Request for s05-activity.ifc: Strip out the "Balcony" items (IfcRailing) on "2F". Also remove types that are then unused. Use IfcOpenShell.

First a look at what the model holds.

```python
import ifcopenshell
import ifcopenshell.util.element

model = ifcopenshell.open("s05-activity.ifc")
print(model.schema)
storey = next(s for s in model.by_type("IfcBuildingStorey") if s.Name == "2F")
railings = [e for e in ifcopenshell.util.element.get_decomposition(storey) if e.is_a("IfcRailing")]
seen = {}
for e in railings:
    element_type = ifcopenshell.util.element.get_type(e)
    name = element_type.Name if element_type not in (None, e) else None
    seen[name] = seen.get(name, 0) + 1
for name, count in sorted(seen.items(), key=str):
    print(count, "x", name)
```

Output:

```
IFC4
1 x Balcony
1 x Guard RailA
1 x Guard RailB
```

```python
import ifcopenshell
import ifcopenshell.api.root
import ifcopenshell.util.element

model = ifcopenshell.open("s05-activity.ifc")

storey = next(s for s in model.by_type("IfcBuildingStorey") if s.Name == "2F")
railings = [e for e in ifcopenshell.util.element.get_decomposition(storey) if e.is_a("IfcRailing")]
targets = [e for e in railings if (t := ifcopenshell.util.element.get_type(e)) not in (None, e) and t.Name == "Balcony"]
types = {ifcopenshell.util.element.get_type(e) for e in targets} - {None, *targets}

for e in targets:
    ifcopenshell.api.root.remove_product(model, product=e)
print(len(targets), "removed")

unused = [t for t in types if not ifcopenshell.util.element.get_types(t)]
for t in unused:
    ifcopenshell.api.root.remove_product(model, product=t)
print(len(unused), "unused types removed")

model.write("s05-activity_v2.ifc")
```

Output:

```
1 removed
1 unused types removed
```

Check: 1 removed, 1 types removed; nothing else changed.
